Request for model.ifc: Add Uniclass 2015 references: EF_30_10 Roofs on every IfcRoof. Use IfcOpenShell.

First a look at what the model holds.

```python
import ifcopenshell

model = ifcopenshell.open("model.ifc")
print(model.schema)
print("classifications:", [c.Name for c in model.by_type("IfcClassification")])
for ifc_class in ("IfcDoor", "IfcRoof", "IfcStair", "IfcWall", "IfcWindow"):
    print(ifc_class, len(model.by_type(ifc_class)))
```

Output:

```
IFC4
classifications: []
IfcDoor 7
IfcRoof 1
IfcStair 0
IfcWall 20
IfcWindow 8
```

```python
import ifcopenshell
import ifcopenshell.api.classification

model = ifcopenshell.open("model.ifc")

system = ifcopenshell.api.classification.add_classification(model, classification="Uniclass 2015")

codes = {
    "IfcRoof": ("EF_30_10", "Roofs"),
}
for ifc_class, (code, name) in codes.items():
    products = model.by_type(ifc_class)
    ifcopenshell.api.classification.add_reference(
        model, products=products, classification=system, identification=code, name=name
    )
    print(code, len(products))

model.write("model_v2.ifc")
```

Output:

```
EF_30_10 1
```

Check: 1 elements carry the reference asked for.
